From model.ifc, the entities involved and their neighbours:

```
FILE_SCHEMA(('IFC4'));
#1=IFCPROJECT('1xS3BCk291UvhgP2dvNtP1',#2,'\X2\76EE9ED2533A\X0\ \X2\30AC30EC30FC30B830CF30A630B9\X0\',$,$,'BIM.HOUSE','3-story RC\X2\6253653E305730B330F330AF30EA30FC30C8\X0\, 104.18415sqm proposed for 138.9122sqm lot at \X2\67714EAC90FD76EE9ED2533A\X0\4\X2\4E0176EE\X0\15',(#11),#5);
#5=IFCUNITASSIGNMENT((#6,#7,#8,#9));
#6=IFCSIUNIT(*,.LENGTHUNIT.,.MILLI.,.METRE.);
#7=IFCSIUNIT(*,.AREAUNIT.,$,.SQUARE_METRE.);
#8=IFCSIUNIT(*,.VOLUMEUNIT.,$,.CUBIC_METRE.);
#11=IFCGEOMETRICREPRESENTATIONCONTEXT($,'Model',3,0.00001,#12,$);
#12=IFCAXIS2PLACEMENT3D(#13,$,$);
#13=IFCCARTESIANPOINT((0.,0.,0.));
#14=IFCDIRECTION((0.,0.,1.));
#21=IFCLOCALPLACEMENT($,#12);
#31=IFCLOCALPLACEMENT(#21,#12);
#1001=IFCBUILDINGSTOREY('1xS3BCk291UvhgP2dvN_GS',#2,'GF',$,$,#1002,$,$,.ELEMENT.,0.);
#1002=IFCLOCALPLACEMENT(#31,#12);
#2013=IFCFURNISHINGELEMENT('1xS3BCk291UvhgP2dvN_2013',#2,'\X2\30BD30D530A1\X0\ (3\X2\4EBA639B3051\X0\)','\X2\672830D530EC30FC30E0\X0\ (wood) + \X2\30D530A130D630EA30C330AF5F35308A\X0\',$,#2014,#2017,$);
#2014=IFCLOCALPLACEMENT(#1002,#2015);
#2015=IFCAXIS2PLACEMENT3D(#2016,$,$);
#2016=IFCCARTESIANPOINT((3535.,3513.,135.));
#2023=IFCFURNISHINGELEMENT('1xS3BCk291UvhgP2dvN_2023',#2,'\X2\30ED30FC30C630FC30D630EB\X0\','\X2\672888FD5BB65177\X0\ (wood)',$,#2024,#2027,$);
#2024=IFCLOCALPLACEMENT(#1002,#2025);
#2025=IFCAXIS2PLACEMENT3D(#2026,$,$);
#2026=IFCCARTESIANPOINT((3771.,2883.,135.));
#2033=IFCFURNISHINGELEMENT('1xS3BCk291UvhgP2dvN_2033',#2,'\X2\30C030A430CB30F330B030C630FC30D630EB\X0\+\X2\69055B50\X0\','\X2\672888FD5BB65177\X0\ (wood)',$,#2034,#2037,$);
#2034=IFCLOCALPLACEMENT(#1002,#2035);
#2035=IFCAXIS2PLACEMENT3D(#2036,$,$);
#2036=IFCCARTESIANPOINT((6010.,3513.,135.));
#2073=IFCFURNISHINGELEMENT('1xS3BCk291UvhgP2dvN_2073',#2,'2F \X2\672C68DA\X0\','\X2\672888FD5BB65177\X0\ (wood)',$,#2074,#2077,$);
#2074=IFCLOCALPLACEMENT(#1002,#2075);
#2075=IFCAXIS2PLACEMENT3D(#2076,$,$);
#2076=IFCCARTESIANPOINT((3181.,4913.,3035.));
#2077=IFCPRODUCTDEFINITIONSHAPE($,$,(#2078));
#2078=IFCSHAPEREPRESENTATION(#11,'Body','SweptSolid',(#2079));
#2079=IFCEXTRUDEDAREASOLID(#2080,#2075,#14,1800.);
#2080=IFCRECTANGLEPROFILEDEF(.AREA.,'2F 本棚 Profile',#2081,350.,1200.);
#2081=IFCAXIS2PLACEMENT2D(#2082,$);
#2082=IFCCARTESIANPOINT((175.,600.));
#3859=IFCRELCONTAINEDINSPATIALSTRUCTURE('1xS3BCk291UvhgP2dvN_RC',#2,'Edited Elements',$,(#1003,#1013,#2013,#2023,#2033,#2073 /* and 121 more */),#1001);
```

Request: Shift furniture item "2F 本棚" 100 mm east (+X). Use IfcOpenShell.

```python
import ifcopenshell
import ifcopenshell.api.geometry
import ifcopenshell.util.placement

model = ifcopenshell.open("model.ifc")

item = model.by_guid("1xS3BCk291UvhgP2dvN_2073")
matrix = ifcopenshell.util.placement.get_local_placement(item.ObjectPlacement)
matrix[0, 3] += 100.0
ifcopenshell.api.geometry.edit_object_placement(model, product=item, matrix=matrix, is_si=False)

print(ifcopenshell.util.placement.get_local_placement(item.ObjectPlacement).round(3) + 0.0)

model.write("model-out.ifc")
```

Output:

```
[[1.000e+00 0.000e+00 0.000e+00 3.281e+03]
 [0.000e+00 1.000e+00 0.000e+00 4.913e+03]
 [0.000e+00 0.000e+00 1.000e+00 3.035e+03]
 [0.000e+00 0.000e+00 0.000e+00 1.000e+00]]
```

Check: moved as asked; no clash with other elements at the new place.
